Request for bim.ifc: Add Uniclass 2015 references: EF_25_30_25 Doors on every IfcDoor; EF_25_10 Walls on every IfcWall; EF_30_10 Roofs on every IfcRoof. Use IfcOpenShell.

First a look at what the model holds.

```python
import ifcopenshell

model = ifcopenshell.open("bim.ifc")
print(model.schema)
print("classifications:", [c.Name for c in model.by_type("IfcClassification")])
for ifc_class in ("IfcDoor", "IfcRoof", "IfcStair", "IfcWall", "IfcWindow"):
    print(ifc_class, len(model.by_type(ifc_class)))
```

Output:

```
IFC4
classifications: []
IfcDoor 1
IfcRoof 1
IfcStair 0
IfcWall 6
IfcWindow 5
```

```python
import ifcopenshell
import ifcopenshell.api.classification

model = ifcopenshell.open("bim.ifc")

system = ifcopenshell.api.classification.add_classification(model, classification="Uniclass 2015")

codes = {
    "IfcDoor": ("EF_25_30_25", "Doors"),
    "IfcWall": ("EF_25_10", "Walls"),
    "IfcRoof": ("EF_30_10", "Roofs"),
}
for ifc_class, (code, name) in codes.items():
    products = model.by_type(ifc_class)
    ifcopenshell.api.classification.add_reference(
        model, products=products, classification=system, identification=code, name=name
    )
    print(code, len(products))

model.write("bim_edited.ifc")
```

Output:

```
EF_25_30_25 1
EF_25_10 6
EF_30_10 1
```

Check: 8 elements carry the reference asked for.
